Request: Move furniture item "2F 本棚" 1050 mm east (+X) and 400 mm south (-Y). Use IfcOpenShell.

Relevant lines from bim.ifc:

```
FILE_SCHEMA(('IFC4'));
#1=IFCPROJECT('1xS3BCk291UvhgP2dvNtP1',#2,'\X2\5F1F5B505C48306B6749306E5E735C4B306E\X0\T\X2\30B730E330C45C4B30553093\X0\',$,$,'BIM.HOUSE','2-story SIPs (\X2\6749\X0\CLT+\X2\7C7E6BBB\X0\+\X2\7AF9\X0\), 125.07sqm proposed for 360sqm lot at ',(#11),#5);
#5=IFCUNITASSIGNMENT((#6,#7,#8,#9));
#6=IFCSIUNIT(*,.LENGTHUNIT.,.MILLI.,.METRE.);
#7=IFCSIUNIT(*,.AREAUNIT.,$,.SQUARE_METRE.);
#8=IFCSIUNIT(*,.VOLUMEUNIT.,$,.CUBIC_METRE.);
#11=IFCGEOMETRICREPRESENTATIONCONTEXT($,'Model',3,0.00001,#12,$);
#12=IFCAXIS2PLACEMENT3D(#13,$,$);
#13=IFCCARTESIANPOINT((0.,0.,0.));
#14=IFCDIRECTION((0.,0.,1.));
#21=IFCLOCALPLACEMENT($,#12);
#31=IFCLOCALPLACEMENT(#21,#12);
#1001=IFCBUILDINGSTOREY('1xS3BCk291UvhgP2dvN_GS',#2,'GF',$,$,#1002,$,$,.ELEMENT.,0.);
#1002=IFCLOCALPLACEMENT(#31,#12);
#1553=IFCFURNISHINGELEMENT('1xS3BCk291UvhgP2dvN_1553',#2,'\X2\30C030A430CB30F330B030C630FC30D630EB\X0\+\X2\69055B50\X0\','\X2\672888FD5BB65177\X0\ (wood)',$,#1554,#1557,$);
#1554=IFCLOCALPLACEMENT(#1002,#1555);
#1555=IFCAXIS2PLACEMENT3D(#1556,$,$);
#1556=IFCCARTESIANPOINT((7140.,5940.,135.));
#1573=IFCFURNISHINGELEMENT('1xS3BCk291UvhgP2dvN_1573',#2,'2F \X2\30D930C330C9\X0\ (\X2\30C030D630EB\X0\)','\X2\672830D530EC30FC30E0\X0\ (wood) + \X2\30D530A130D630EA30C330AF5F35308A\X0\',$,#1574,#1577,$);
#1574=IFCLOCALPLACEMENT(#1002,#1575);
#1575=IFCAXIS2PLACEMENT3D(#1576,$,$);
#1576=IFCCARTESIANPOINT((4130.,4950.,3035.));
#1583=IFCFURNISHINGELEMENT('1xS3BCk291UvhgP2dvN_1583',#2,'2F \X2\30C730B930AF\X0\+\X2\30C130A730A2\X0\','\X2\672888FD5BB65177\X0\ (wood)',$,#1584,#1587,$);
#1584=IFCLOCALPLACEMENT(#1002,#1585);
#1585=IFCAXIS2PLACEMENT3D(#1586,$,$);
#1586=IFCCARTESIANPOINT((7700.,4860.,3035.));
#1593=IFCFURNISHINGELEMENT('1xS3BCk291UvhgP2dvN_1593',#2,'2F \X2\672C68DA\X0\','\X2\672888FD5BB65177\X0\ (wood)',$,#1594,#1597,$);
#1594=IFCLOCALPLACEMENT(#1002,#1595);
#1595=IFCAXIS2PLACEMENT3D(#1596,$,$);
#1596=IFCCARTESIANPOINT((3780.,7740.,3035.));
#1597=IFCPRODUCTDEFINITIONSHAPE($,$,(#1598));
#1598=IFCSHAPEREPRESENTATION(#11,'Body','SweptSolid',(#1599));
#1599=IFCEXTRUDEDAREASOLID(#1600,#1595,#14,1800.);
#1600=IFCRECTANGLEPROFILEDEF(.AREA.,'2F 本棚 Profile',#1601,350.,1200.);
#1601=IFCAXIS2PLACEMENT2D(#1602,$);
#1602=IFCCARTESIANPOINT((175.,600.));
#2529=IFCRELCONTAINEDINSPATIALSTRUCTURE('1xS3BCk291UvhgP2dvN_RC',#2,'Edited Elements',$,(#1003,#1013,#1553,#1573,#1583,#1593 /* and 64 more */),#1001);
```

```python
import ifcopenshell
import ifcopenshell.api.geometry
import ifcopenshell.util.placement

model = ifcopenshell.open("bim.ifc")

item = model.by_id(1593)
matrix = ifcopenshell.util.placement.get_local_placement(item.ObjectPlacement)
matrix[0, 3] += 1050.0
matrix[1, 3] -= 400.0
ifcopenshell.api.geometry.edit_object_placement(model, product=item, matrix=matrix, is_si=False)

print(ifcopenshell.util.placement.get_local_placement(item.ObjectPlacement).round(3) + 0.0)

model.write("bim_updated.ifc")
```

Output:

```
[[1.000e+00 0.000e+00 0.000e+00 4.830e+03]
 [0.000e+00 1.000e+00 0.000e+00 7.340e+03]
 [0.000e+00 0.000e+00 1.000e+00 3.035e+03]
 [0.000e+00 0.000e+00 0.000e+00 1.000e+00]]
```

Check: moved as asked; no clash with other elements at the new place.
